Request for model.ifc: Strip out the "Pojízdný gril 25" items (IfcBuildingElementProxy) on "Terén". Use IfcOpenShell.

First a look at what the model holds.

```python
import ifcopenshell
import ifcopenshell.util.element

model = ifcopenshell.open("model.ifc")
print(model.schema)
storey = next(s for s in model.by_type("IfcBuildingStorey") if s.Name == "Terén")
proxies = [e for e in ifcopenshell.util.element.get_decomposition(storey) if e.is_a("IfcBuildingElementProxy")]
seen = {}
for e in proxies:
    element_type = ifcopenshell.util.element.get_type(e)
    name = element_type.Name if element_type not in (None, e) else None
    seen[name] = seen.get(name, 0) + 1
for name, count in sorted(seen.items(), key=str):
    print(count, "x", name)
```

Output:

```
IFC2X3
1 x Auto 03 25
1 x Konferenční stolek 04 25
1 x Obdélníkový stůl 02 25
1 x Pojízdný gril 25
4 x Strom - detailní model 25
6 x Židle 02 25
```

```python
import ifcopenshell
import ifcopenshell.api.root
import ifcopenshell.util.element

model = ifcopenshell.open("model.ifc")

storey = next(s for s in model.by_type("IfcBuildingStorey") if s.Name == "Terén")
proxies = [e for e in ifcopenshell.util.element.get_decomposition(storey) if e.is_a("IfcBuildingElementProxy")]
targets = [e for e in proxies if (t := ifcopenshell.util.element.get_type(e)) not in (None, e) and t.Name == "Pojízdný gril 25"]

for e in targets:
    ifcopenshell.api.root.remove_product(model, product=e)
print(len(targets), "removed")

model.write("model_rev.ifc")
```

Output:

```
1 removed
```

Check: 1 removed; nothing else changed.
